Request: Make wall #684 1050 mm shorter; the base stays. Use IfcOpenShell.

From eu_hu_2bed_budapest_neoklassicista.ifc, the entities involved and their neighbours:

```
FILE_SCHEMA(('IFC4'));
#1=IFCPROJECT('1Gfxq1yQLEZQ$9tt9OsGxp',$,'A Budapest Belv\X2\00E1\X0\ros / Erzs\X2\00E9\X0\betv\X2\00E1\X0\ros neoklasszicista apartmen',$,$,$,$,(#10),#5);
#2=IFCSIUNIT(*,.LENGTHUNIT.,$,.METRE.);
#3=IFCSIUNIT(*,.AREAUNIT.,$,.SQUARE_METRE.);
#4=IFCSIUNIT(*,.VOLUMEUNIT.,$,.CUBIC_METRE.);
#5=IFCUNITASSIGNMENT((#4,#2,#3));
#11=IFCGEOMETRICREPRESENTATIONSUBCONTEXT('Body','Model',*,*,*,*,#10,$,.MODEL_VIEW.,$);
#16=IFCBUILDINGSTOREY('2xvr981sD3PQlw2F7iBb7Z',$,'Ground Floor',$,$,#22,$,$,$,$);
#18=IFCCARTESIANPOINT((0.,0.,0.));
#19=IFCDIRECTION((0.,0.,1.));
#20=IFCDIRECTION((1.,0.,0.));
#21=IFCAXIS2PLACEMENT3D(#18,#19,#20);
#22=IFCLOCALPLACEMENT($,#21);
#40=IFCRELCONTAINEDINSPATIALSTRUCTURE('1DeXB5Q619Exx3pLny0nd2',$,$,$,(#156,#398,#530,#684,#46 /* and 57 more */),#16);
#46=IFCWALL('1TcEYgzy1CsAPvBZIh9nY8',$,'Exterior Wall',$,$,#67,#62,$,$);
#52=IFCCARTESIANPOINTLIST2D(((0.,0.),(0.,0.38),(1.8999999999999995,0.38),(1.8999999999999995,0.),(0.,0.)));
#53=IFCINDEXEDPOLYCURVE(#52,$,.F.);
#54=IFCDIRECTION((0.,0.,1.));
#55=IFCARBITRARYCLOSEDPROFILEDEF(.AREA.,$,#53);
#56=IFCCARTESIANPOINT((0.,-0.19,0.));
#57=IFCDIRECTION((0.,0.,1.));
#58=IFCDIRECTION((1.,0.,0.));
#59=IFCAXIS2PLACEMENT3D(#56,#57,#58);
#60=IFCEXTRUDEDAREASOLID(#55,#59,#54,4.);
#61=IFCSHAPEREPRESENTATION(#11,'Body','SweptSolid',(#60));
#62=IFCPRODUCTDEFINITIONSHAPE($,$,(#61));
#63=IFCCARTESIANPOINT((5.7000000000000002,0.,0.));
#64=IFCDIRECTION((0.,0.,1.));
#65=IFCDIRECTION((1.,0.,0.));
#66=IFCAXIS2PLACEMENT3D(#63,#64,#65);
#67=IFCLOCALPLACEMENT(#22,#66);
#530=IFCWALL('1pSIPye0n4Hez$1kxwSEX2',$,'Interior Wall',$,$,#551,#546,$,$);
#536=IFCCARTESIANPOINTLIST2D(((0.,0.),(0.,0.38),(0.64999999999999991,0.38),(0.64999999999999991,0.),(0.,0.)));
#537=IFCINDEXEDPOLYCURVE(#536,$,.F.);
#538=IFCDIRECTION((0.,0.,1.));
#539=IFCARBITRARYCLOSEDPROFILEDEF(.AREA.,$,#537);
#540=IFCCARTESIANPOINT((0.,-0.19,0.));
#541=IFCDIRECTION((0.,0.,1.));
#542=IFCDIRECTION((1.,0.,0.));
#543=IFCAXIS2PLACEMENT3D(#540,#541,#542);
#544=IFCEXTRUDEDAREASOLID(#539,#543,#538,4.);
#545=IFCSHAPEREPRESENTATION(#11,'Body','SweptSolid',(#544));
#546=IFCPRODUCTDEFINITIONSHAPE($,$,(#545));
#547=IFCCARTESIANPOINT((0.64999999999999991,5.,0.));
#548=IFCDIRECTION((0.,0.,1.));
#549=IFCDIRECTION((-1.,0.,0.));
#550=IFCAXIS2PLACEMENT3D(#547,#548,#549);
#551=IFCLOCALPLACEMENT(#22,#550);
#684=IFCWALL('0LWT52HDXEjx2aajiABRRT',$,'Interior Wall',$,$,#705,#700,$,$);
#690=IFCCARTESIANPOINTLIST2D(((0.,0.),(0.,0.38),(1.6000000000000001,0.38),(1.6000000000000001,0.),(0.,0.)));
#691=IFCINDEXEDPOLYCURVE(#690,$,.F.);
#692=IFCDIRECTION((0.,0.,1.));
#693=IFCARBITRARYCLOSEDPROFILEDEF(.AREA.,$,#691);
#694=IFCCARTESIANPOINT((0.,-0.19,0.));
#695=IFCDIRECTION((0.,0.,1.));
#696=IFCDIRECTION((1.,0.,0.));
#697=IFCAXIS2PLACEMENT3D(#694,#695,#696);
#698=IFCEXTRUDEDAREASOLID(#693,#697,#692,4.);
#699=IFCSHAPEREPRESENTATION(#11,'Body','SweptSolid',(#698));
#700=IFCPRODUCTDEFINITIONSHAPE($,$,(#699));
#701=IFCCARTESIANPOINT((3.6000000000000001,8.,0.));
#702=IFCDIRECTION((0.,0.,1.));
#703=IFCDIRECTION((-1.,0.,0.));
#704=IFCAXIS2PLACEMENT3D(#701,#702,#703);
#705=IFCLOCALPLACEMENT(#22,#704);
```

```python
import ifcopenshell
import ifcopenshell.geom
import ifcopenshell.util.representation
import ifcopenshell.util.shape
import ifcopenshell.util.unit

model = ifcopenshell.open("eu_hu_2bed_budapest_neoklassicista.ifc")
unit_scale = ifcopenshell.util.unit.calculate_unit_scale(model)
settings = ifcopenshell.geom.settings()


def volume(element):
    """Net volume in cubic metres, openings subtracted."""
    shape = ifcopenshell.geom.create_shape(settings, element)
    return ifcopenshell.util.shape.get_volume(shape.geometry)


wall = model.by_guid("0LWT52HDXEjx2aajiABRRT")
before = volume(wall)

body = ifcopenshell.util.representation.get_representation(wall, "Model", "Body")
solid = body.Items[0]
old_height = solid.Depth
solid.Depth -= 1.05 / unit_scale
after = volume(wall)

print(f"height {old_height:g} -> {solid.Depth:g}, volume {before:.3f} -> {after:.3f} m3")

model.write("eu_hu_2bed_budapest_neoklassicista_edited.ifc")
```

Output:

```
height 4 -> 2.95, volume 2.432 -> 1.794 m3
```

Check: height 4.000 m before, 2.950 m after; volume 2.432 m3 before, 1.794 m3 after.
